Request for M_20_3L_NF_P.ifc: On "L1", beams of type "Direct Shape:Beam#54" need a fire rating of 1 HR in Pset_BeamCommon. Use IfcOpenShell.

First a look at what the model holds.

```python
import ifcopenshell
import ifcopenshell.util.element

model = ifcopenshell.open("M_20_3L_NF_P.ifc")
print(model.schema)
storey = next(s for s in model.by_type("IfcBuildingStorey") if s.Name == "L1")
beams = [e for e in ifcopenshell.util.element.get_decomposition(storey) if e.is_a("IfcBeam")]
seen = {}
for e in beams:
    element_type = ifcopenshell.util.element.get_type(e)
    key = (element_type.Name if element_type != e and element_type else None, ifcopenshell.util.element.get_pset(e, "Pset_BeamCommon", "FireRating"))
    seen[key] = seen.get(key, 0) + 1
for (name, value), count in sorted(seen.items(), key=str):
    print(count, "x", name, "|", value)
```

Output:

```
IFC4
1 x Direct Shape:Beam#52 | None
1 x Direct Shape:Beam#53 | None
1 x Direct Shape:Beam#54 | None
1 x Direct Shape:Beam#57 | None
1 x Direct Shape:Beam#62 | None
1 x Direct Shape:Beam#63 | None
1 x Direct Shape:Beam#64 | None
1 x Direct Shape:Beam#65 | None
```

```python
import ifcopenshell
import ifcopenshell.api.pset
import ifcopenshell.util.element

model = ifcopenshell.open("M_20_3L_NF_P.ifc")

storey = next(s for s in model.by_type("IfcBuildingStorey") if s.Name == "L1")
beams = [e for e in ifcopenshell.util.element.get_decomposition(storey) if e.is_a("IfcBeam")]

count = 0
for e in beams:
    element_type = ifcopenshell.util.element.get_type(e)
    if element_type in (None, e) or element_type.Name != "Direct Shape:Beam#54":
        continue
    # add_pset returns the element's existing set when there is one.
    pset = ifcopenshell.api.pset.add_pset(model, product=e, name="Pset_BeamCommon")
    ifcopenshell.api.pset.edit_pset(model, pset=pset, properties={"FireRating": "1 HR"})
    count += 1

print(count, "beams updated")

model.write("M_20_3L_NF_P_v2.ifc")
```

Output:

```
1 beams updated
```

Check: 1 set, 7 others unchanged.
